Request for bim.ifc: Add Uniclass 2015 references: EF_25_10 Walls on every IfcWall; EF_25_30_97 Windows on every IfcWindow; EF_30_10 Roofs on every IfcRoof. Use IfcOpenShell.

First a look at what the model holds.

```python
import ifcopenshell

model = ifcopenshell.open("bim.ifc")
print(model.schema)
print("classifications:", [c.Name for c in model.by_type("IfcClassification")])
for ifc_class in ("IfcDoor", "IfcRoof", "IfcStair", "IfcWall", "IfcWindow"):
    print(ifc_class, len(model.by_type(ifc_class)))
```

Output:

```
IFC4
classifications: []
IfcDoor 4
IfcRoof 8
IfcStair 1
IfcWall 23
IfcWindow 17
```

```python
import ifcopenshell
import ifcopenshell.api.classification

model = ifcopenshell.open("bim.ifc")

system = ifcopenshell.api.classification.add_classification(model, classification="Uniclass 2015")

codes = {
    "IfcWall": ("EF_25_10", "Walls"),
    "IfcWindow": ("EF_25_30_97", "Windows"),
    "IfcRoof": ("EF_30_10", "Roofs"),
}
for ifc_class, (code, name) in codes.items():
    products = model.by_type(ifc_class)
    ifcopenshell.api.classification.add_reference(
        model, products=products, classification=system, identification=code, name=name
    )
    print(code, len(products))

model.write("bim_rev.ifc")
```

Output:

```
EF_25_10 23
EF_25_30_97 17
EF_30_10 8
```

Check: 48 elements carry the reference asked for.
